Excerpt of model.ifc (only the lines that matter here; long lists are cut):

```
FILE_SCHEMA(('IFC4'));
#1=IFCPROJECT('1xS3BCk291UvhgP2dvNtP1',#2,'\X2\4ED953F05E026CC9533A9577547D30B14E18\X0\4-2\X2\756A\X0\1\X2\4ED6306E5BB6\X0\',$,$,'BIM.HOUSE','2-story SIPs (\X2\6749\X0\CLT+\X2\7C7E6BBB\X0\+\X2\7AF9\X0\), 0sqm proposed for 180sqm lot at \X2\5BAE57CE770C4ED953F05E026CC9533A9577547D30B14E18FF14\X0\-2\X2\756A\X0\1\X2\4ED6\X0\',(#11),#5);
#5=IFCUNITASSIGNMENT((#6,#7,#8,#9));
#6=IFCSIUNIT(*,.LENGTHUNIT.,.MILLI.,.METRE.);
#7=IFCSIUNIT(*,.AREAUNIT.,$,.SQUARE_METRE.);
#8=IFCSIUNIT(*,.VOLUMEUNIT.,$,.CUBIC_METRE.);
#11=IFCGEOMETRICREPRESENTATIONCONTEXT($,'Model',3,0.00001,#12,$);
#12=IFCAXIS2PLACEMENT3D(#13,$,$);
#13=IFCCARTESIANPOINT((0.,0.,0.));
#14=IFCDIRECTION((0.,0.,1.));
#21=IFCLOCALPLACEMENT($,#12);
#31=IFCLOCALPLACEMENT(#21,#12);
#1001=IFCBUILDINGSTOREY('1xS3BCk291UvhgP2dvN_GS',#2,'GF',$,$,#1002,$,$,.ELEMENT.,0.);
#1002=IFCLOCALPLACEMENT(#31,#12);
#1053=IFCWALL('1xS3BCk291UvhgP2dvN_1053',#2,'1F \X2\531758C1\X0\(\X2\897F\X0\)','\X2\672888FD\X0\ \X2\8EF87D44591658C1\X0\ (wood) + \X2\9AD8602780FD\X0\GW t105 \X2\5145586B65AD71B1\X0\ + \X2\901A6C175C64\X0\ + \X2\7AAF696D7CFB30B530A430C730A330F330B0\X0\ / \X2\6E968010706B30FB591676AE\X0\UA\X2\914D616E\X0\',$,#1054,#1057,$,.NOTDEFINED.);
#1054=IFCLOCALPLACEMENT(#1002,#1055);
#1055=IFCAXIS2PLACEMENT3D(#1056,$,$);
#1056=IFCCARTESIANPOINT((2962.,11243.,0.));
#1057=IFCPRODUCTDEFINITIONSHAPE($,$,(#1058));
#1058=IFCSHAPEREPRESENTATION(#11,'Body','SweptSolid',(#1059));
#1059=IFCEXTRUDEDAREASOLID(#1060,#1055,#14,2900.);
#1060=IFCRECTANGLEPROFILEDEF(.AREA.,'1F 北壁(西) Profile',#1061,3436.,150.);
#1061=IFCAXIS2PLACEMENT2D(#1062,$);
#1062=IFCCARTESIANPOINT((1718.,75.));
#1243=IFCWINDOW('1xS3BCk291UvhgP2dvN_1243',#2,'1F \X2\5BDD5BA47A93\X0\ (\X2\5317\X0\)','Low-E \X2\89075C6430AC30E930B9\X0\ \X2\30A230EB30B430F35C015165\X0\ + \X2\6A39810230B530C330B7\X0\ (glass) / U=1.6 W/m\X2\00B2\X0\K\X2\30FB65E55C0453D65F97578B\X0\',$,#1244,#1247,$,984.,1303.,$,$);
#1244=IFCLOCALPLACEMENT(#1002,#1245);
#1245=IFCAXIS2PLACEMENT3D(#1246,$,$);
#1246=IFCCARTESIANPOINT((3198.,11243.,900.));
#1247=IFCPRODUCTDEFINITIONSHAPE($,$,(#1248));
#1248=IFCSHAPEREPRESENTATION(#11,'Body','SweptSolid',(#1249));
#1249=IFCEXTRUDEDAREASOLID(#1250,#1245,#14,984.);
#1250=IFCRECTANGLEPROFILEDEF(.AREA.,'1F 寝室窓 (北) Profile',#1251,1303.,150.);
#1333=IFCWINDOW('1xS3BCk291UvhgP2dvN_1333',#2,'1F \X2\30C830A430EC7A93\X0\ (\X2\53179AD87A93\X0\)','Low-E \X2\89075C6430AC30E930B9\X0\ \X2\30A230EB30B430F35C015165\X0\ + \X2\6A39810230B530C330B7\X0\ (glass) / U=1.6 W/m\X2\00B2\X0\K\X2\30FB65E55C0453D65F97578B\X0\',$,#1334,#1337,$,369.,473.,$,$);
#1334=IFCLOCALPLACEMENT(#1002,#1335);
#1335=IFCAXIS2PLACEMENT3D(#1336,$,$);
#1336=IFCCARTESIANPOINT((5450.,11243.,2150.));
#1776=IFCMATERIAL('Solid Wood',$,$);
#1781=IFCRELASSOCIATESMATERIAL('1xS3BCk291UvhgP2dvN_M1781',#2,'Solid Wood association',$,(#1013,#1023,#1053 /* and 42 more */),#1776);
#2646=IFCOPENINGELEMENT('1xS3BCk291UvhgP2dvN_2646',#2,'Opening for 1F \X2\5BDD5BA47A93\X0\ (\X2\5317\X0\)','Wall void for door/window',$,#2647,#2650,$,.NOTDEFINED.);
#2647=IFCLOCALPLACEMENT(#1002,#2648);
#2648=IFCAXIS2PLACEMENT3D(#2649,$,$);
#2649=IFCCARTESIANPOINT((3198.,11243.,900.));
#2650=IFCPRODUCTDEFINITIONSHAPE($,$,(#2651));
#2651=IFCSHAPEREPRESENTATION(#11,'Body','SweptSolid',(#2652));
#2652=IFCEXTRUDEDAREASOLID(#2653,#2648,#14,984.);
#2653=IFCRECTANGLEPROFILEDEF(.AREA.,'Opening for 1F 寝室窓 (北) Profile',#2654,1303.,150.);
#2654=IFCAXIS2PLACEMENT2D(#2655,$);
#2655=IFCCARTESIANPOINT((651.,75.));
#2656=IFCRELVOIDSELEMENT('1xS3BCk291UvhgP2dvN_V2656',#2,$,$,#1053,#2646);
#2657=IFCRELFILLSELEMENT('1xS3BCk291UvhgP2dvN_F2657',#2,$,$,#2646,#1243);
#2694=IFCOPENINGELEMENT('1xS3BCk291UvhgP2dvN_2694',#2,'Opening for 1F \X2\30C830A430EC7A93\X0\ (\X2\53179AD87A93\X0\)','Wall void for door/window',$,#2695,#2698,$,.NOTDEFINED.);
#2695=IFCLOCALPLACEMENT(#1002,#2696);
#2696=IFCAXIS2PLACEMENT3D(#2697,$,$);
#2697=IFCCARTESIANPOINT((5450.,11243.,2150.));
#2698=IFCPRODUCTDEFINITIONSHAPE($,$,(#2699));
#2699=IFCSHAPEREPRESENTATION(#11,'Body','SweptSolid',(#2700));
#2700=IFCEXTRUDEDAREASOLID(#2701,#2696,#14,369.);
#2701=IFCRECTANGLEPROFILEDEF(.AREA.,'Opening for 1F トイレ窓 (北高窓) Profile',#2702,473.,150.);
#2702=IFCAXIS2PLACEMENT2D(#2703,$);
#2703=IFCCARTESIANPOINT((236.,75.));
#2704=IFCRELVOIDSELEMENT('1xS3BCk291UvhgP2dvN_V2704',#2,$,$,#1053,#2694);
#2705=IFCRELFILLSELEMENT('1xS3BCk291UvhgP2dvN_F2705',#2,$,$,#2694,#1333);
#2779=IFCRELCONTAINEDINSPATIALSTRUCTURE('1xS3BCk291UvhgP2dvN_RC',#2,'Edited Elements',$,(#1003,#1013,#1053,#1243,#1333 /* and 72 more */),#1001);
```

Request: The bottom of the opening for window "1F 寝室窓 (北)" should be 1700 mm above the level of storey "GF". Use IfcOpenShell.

```python
import numpy as np
import ifcopenshell
import ifcopenshell.api.geometry
import ifcopenshell.geom
import ifcopenshell.util.element
import ifcopenshell.util.placement
import ifcopenshell.util.shape
import ifcopenshell.util.unit

model = ifcopenshell.open("model.ifc")
unit_scale = ifcopenshell.util.unit.calculate_unit_scale(model)

window = model.by_id(1243)
opening = window.FillsVoids[0].RelatingOpeningElement
storey = ifcopenshell.util.element.get_container(window, ifc_class="IfcBuildingStorey")
level = ifcopenshell.util.placement.get_local_placement(storey.ObjectPlacement)[2, 3]

# The opening's origin need not be at the sill, so measure its lowest point.
shape = ifcopenshell.geom.create_shape(ifcopenshell.geom.settings(), opening)
bottom = ifcopenshell.util.shape.get_shape_bottom_elevation(shape, shape.geometry) / unit_scale
dz = level + 1700.0 - bottom

shift = np.array([0.0, 0.0, dz])
# The window is not placed relative to its opening, so move both.
for product in (opening, window):
    matrix = ifcopenshell.util.placement.get_local_placement(product.ObjectPlacement)
    matrix[:3, 3] += shift
    ifcopenshell.api.geometry.edit_object_placement(model, product=product, matrix=matrix, is_si=False)

print(f"moved by {dz * unit_scale:+.3f} m")

model.write("model_v2.ifc")
```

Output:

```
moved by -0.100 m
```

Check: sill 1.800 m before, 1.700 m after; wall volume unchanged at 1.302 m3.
